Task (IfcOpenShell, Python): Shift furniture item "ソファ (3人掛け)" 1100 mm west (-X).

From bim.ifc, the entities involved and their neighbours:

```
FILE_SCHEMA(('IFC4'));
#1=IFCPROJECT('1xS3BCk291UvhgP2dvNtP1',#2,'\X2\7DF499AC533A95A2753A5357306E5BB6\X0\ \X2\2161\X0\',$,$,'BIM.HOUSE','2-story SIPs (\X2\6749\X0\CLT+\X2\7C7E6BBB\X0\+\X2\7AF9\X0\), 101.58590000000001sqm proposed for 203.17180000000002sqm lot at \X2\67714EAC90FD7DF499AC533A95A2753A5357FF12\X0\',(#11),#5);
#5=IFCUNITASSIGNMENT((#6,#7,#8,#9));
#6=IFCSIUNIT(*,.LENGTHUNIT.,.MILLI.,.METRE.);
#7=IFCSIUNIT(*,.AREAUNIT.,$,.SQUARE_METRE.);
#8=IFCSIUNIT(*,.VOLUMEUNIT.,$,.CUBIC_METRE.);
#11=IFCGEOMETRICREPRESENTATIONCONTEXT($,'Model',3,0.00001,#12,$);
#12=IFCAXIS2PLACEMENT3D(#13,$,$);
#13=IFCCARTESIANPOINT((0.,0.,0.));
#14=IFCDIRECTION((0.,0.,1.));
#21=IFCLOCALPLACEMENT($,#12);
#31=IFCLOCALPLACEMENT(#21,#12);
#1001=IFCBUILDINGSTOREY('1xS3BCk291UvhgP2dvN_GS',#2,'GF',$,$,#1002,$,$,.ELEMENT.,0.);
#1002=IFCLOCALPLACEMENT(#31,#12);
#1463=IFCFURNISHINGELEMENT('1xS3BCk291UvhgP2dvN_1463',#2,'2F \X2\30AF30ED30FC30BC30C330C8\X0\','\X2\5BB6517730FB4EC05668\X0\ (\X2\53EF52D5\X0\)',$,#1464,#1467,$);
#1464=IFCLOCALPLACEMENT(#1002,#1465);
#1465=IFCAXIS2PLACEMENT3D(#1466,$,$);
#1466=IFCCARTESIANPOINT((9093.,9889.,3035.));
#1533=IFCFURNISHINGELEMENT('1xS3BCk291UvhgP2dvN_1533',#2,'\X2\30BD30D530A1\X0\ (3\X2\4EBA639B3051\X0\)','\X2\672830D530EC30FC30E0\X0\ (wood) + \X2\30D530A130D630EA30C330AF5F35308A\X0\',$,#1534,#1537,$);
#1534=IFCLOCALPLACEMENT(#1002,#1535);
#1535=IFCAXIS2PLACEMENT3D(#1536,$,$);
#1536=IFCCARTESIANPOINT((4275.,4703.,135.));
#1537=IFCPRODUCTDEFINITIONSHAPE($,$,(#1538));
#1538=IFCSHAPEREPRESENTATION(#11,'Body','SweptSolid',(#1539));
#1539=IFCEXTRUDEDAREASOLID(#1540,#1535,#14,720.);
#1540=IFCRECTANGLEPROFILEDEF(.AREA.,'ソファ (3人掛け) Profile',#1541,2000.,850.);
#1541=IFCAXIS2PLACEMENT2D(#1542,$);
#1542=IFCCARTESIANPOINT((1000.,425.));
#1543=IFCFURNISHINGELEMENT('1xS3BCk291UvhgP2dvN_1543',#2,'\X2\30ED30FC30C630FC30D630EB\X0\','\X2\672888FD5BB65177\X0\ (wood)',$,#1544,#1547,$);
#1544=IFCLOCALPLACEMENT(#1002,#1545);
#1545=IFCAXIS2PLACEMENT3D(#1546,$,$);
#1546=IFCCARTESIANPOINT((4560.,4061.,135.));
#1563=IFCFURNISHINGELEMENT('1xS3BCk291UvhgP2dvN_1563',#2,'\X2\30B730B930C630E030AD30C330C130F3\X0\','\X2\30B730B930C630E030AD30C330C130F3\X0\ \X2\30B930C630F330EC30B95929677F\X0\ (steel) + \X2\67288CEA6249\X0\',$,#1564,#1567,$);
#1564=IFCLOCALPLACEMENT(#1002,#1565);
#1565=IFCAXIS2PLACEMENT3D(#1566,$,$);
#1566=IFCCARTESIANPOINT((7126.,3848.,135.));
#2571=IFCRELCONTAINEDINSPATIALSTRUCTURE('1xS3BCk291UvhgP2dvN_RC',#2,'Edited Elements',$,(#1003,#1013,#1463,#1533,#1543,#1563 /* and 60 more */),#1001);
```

```python
import ifcopenshell
import ifcopenshell.api.geometry
import ifcopenshell.util.placement
import ifcopenshell.util.unit

model = ifcopenshell.open("bim.ifc")
unit_scale = ifcopenshell.util.unit.calculate_unit_scale(model)

item = model.by_guid("1xS3BCk291UvhgP2dvN_1533")
matrix = ifcopenshell.util.placement.get_local_placement(item.ObjectPlacement)
matrix[0, 3] -= 1.1 / unit_scale
ifcopenshell.api.geometry.edit_object_placement(model, product=item, matrix=matrix, is_si=False)

print(ifcopenshell.util.placement.get_local_placement(item.ObjectPlacement).round(3) + 0.0)

model.write("bim_v2.ifc")
```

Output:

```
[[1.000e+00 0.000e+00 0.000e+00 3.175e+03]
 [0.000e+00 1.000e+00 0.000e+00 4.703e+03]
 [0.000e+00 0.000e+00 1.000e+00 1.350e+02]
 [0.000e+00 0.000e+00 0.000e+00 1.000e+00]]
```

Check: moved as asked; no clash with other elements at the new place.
